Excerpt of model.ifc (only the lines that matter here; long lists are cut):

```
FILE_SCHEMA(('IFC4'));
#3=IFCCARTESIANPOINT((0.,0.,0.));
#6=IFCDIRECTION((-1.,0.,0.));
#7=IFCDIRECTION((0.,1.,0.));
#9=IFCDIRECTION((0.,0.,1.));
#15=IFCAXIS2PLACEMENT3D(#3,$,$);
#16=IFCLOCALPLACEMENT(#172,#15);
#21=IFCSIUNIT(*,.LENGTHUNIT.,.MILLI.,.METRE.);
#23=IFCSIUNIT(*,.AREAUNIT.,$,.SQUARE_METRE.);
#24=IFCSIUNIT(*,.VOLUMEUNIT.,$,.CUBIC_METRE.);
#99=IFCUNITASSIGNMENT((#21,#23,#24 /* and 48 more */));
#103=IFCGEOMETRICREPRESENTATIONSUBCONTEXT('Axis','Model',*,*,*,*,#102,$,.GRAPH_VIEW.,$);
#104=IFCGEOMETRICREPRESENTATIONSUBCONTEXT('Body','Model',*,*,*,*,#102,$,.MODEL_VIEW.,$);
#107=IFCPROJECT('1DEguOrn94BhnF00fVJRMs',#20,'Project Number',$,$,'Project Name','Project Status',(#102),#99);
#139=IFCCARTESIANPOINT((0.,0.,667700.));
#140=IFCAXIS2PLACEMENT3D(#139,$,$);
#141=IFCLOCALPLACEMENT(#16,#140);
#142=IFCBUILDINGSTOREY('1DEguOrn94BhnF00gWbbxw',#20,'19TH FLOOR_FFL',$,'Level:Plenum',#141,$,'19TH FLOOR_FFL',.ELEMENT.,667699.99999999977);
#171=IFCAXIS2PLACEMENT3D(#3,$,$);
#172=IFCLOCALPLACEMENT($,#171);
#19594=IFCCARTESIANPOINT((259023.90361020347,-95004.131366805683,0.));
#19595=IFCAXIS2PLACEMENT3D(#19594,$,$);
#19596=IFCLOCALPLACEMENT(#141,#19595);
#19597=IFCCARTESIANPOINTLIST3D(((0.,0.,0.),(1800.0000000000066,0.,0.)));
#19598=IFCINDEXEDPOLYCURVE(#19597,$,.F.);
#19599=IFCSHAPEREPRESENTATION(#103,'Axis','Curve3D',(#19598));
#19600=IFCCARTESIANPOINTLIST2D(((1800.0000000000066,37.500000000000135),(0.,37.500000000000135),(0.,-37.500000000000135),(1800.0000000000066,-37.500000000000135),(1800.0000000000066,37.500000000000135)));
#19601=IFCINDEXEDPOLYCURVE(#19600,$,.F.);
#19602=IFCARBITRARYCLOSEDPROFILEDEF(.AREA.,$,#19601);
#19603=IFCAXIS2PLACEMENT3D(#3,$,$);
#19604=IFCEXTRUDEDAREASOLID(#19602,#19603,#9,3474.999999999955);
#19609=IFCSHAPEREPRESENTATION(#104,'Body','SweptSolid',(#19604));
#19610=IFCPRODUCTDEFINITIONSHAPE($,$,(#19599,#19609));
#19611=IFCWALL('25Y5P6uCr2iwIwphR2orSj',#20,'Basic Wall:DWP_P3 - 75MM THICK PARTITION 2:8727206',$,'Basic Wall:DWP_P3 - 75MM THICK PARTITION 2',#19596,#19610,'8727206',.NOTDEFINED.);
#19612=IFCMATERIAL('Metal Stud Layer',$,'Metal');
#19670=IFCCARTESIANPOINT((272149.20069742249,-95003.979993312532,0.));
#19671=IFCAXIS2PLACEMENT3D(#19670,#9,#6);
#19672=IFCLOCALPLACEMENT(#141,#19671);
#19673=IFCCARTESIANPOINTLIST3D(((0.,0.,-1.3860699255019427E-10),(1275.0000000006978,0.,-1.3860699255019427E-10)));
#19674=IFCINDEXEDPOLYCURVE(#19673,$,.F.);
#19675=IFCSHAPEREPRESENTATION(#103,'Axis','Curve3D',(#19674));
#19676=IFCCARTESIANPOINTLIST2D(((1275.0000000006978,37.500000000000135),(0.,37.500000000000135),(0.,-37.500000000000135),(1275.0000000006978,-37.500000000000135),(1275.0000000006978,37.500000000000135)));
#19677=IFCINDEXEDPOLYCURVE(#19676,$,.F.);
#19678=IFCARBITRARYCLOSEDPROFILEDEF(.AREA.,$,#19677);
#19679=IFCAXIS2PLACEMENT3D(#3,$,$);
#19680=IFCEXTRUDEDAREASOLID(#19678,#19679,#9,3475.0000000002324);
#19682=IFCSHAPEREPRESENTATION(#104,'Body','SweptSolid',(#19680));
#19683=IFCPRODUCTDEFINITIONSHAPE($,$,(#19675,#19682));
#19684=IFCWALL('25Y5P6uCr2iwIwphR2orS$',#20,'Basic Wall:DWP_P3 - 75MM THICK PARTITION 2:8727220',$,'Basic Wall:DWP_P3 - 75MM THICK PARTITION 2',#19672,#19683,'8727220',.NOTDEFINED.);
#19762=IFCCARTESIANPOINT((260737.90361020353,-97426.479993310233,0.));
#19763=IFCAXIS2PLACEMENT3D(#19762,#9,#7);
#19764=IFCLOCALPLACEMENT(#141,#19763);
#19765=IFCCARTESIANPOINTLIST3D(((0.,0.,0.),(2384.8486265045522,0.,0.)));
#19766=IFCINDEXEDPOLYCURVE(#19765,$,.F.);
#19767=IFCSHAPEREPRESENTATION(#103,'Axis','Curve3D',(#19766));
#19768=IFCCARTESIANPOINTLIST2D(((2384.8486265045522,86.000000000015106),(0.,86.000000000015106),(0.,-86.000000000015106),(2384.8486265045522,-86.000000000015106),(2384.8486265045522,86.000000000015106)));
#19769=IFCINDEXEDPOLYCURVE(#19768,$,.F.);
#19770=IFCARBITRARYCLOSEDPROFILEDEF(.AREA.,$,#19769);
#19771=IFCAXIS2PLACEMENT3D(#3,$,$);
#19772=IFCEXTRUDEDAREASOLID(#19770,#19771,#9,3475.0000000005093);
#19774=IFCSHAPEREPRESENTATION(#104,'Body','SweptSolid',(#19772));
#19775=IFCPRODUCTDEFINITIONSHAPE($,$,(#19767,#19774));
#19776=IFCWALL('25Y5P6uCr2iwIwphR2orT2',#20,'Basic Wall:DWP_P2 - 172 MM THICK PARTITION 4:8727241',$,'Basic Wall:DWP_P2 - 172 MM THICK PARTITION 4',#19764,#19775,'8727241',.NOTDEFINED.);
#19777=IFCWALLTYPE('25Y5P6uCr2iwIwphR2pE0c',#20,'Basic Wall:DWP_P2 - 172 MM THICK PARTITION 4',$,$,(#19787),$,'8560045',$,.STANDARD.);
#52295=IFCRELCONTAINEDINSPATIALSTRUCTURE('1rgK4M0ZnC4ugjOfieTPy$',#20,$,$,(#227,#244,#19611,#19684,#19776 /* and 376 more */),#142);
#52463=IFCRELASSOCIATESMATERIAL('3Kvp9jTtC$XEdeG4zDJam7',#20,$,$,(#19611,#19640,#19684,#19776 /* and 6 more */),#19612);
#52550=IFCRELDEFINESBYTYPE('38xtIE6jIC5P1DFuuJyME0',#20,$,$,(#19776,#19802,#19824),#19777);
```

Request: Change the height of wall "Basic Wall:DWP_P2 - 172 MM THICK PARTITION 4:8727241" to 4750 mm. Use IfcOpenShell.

```python
import ifcopenshell
import ifcopenshell.geom
import ifcopenshell.util.representation
import ifcopenshell.util.shape

model = ifcopenshell.open("model.ifc")
settings = ifcopenshell.geom.settings()


def volume(element):
    """Net volume in cubic metres, openings subtracted."""
    shape = ifcopenshell.geom.create_shape(settings, element)
    return ifcopenshell.util.shape.get_volume(shape.geometry)


wall = model.by_id(19776)
before = volume(wall)

body = ifcopenshell.util.representation.get_representation(wall, "Model", "Body")
solid = body.Items[0]
old_height = solid.Depth
solid.Depth = 4750.0
after = volume(wall)

print(f"height {old_height:g} -> {solid.Depth:g}, volume {before:.3f} -> {after:.3f} m3")

model.write("model_rev.ifc")
```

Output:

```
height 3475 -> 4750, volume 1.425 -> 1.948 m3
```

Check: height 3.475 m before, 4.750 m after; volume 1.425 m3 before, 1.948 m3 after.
